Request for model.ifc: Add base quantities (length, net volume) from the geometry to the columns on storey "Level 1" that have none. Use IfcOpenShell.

First a look at what the model holds.

```python
import ifcopenshell
import ifcopenshell.util.element
import ifcopenshell.util.unit

model = ifcopenshell.open("model.ifc")
print(model.schema)
for unit_type in ("LENGTHUNIT", "AREAUNIT", "VOLUMEUNIT"):
    print(unit_type, ifcopenshell.util.unit.calculate_unit_scale(model, unit_type))
storey = next(s for s in model.by_type("IfcBuildingStorey") if s.Name == "Level 1")
columns = [e for e in ifcopenshell.util.element.get_decomposition(storey) if e.is_a("IfcColumn")]
for e in sorted(columns, key=lambda e: e.id()):
    print(e.id(), e.is_a(), e.Name, list(ifcopenshell.util.element.get_psets(e, qtos_only=True)), sep=" | ")
```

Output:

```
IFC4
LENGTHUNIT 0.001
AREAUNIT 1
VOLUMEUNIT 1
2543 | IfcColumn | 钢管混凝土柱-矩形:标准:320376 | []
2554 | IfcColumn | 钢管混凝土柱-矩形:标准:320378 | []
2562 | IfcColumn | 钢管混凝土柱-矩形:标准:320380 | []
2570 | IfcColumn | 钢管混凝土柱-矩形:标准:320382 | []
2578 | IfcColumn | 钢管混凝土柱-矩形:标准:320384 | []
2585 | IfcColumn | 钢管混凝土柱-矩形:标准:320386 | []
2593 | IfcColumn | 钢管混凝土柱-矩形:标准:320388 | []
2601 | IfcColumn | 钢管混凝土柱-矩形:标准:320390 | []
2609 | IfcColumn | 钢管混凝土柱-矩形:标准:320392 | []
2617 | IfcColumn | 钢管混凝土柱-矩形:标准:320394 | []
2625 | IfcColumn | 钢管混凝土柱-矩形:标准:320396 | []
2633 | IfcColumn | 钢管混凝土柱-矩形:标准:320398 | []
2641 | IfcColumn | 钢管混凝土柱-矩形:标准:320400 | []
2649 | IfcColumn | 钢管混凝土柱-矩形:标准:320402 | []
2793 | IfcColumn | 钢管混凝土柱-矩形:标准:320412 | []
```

```python
import ifcopenshell
import ifcopenshell.api.pset
import ifcopenshell.geom
import ifcopenshell.util.element
import ifcopenshell.util.shape
import ifcopenshell.util.unit

model = ifcopenshell.open("model.ifc")
unit_scale = ifcopenshell.util.unit.calculate_unit_scale(model)
volume_scale = ifcopenshell.util.unit.calculate_unit_scale(model, "VOLUMEUNIT")
settings = ifcopenshell.geom.settings()

storey = next(s for s in model.by_type("IfcBuildingStorey") if s.Name == "Level 1")
columns = [e for e in ifcopenshell.util.element.get_decomposition(storey) if e.is_a("IfcColumn")]

for e in sorted(columns, key=lambda e: e.id()):
    if ifcopenshell.util.element.get_psets(e, qtos_only=True, should_inherit=False):
        continue
    # Geometry comes back in metres, in the element's own axes.
    shape = ifcopenshell.geom.create_shape(settings, e)
    values = {
        "Length": ifcopenshell.util.shape.get_z(shape.geometry) / unit_scale,
        "NetVolume": ifcopenshell.util.shape.get_volume(shape.geometry) / volume_scale,
    }
    qto = ifcopenshell.api.pset.add_qto(model, product=e, name="Qto_ColumnBaseQuantities")
    ifcopenshell.api.pset.edit_qto(model, qto=qto, properties=values)
    print(e.id(), {k: round(v, 3) for k, v in values.items()})

model.write("model_rev.ifc")
```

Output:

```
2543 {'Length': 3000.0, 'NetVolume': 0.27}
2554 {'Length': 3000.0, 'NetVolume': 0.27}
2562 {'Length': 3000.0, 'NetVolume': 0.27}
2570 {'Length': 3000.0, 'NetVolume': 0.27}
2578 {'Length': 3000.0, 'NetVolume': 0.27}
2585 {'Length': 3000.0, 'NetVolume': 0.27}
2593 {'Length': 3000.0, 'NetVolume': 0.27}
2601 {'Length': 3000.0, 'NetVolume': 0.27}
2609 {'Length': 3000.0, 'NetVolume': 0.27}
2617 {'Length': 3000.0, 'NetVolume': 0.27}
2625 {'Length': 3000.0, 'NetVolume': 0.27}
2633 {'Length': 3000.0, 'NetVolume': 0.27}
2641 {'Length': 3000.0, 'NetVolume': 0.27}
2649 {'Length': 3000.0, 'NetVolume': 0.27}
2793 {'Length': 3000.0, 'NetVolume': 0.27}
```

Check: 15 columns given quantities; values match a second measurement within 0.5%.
